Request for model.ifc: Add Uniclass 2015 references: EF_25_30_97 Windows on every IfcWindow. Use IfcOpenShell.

First a look at what the model holds.

```python
import ifcopenshell

model = ifcopenshell.open("model.ifc")
print(model.schema)
print("classifications:", [c.Name for c in model.by_type("IfcClassification")])
for ifc_class in ("IfcDoor", "IfcRoof", "IfcStair", "IfcWall", "IfcWindow"):
    print(ifc_class, len(model.by_type(ifc_class)))
```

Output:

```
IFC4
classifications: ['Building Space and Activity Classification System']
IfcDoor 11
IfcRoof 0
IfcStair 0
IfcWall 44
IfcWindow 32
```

```python
import ifcopenshell
import ifcopenshell.api.classification

model = ifcopenshell.open("model.ifc")

system = ifcopenshell.api.classification.add_classification(model, classification="Uniclass 2015")

codes = {
    "IfcWindow": ("EF_25_30_97", "Windows"),
}
for ifc_class, (code, name) in codes.items():
    products = model.by_type(ifc_class)
    ifcopenshell.api.classification.add_reference(
        model, products=products, classification=system, identification=code, name=name
    )
    print(code, len(products))

model.write("model_edited.ifc")
```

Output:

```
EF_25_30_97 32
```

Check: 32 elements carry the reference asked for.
